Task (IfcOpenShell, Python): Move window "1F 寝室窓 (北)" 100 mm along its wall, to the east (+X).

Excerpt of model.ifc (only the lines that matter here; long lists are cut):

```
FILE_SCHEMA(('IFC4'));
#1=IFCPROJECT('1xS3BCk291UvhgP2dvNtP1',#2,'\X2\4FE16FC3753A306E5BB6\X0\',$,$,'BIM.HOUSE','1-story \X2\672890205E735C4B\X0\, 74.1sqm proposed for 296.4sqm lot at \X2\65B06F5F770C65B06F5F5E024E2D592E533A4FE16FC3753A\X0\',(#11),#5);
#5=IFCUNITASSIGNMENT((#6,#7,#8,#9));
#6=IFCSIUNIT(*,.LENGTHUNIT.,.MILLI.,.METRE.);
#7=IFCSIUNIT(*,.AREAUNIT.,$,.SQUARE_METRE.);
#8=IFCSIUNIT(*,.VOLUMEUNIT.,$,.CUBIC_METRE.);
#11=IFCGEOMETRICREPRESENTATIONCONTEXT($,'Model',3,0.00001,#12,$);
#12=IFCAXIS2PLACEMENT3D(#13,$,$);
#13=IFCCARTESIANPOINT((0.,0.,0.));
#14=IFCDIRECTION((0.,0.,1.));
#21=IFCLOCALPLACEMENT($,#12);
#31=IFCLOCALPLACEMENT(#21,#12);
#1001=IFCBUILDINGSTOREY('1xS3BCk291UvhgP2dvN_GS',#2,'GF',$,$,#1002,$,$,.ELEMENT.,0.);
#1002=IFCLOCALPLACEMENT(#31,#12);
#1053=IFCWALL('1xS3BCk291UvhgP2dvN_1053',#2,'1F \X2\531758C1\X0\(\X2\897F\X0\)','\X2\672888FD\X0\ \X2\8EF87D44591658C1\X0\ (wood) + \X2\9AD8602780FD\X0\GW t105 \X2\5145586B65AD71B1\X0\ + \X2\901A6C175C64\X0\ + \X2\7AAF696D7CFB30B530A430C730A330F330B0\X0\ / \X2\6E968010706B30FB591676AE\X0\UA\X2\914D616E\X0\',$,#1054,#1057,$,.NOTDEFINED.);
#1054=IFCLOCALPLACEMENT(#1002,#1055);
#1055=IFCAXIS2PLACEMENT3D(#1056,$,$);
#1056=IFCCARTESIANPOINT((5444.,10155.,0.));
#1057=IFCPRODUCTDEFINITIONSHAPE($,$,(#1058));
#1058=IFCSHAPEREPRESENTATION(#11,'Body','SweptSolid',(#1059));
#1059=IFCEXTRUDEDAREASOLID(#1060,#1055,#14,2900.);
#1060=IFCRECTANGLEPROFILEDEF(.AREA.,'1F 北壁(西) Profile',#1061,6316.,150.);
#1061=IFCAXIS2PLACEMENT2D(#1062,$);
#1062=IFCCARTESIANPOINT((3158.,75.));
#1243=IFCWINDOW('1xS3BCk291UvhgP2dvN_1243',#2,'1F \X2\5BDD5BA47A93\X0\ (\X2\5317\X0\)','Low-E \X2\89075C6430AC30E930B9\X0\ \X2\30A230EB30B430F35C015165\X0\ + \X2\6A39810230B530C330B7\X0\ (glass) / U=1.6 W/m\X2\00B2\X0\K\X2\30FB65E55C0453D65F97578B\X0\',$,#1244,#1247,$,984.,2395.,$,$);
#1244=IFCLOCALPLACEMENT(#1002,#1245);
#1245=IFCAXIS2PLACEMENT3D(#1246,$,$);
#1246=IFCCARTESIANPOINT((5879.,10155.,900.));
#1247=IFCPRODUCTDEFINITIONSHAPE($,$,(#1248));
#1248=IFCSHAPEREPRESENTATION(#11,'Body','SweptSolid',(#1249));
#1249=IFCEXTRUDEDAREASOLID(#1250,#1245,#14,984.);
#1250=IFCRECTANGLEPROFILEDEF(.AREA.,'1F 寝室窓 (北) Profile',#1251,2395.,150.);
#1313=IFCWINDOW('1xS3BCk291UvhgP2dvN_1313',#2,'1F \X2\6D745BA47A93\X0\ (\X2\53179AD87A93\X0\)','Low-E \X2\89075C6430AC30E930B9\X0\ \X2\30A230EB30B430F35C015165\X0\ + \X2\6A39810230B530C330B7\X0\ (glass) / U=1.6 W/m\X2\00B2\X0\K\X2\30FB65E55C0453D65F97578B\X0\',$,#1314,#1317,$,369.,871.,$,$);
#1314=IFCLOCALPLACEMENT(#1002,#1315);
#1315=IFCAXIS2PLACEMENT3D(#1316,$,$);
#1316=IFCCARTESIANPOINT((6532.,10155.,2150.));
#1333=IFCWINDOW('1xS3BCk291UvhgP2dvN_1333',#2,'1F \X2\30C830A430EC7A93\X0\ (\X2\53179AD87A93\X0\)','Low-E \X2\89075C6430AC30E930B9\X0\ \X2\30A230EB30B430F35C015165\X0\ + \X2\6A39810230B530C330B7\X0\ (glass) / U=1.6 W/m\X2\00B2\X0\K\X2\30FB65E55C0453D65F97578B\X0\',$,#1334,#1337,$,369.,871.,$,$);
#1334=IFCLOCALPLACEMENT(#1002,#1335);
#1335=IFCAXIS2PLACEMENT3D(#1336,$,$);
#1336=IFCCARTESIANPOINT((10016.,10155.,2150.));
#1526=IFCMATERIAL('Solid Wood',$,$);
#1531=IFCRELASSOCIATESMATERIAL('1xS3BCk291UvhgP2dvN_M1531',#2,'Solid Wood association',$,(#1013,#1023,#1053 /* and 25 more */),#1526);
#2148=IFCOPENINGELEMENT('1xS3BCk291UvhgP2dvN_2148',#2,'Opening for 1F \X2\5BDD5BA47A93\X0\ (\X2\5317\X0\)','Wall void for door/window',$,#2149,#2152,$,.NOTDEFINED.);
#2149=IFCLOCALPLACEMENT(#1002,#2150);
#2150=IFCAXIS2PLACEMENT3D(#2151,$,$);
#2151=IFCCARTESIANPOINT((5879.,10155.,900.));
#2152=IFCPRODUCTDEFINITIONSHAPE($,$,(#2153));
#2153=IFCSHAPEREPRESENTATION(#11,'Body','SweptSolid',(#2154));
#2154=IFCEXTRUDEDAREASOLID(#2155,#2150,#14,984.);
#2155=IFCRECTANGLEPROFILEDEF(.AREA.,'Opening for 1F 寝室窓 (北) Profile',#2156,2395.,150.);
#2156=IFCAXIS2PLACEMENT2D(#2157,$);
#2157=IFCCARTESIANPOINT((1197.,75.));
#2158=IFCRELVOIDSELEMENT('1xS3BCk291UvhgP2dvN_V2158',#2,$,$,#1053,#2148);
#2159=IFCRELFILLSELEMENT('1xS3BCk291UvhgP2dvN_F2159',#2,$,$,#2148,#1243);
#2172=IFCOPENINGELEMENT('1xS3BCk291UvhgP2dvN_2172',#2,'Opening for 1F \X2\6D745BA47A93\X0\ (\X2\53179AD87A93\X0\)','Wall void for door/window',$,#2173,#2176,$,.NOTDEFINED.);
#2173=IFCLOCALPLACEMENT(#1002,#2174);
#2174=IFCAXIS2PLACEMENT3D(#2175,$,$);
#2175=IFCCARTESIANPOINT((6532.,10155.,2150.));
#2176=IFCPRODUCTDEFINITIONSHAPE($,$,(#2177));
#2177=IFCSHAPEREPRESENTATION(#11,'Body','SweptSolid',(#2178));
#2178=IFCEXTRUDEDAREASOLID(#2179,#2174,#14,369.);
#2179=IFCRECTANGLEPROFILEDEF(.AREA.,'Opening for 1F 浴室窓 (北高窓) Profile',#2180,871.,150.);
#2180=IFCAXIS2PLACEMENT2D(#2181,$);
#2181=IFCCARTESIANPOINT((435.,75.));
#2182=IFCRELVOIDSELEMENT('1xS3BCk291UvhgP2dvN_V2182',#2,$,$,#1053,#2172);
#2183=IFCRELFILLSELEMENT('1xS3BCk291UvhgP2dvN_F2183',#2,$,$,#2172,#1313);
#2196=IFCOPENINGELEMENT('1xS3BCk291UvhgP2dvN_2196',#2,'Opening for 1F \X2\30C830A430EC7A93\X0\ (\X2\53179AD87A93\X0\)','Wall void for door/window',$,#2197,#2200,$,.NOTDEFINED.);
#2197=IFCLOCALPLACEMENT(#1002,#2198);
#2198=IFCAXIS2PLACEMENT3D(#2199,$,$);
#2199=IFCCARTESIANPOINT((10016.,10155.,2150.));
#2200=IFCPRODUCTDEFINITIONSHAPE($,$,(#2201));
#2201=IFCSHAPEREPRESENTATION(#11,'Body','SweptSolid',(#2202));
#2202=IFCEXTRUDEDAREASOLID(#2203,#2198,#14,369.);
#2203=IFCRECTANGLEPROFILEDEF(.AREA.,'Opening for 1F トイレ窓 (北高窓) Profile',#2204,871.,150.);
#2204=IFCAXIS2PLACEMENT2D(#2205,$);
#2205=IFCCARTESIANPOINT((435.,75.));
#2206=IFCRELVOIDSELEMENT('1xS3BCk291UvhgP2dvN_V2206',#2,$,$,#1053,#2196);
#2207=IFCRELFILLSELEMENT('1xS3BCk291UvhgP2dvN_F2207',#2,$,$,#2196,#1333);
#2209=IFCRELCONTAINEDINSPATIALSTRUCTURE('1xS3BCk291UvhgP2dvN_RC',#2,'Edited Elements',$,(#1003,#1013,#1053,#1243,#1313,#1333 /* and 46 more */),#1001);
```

```python
import ifcopenshell
import ifcopenshell.api.geometry
import ifcopenshell.util.placement
import ifcopenshell.util.unit

model = ifcopenshell.open("model.ifc")
unit_scale = ifcopenshell.util.unit.calculate_unit_scale(model)

window = model.by_id(1243)
opening = window.FillsVoids[0].RelatingOpeningElement
wall = opening.VoidsElements[0].RelatingBuildingElement

wall_matrix = ifcopenshell.util.placement.get_local_placement(wall.ObjectPlacement)
shift = wall_matrix[:3, 0] * 0.1 / unit_scale
before = ifcopenshell.util.placement.get_local_placement(window.ObjectPlacement)[:3, 3].copy()

# The window is not placed relative to its opening, so move both.
for product in (opening, window):
    matrix = ifcopenshell.util.placement.get_local_placement(product.ObjectPlacement)
    matrix[:3, 3] += shift
    ifcopenshell.api.geometry.edit_object_placement(model, product=product, matrix=matrix, is_si=False)

after = ifcopenshell.util.placement.get_local_placement(window.ObjectPlacement)[:3, 3]
print("window moved by", (after - before).round(3) + 0.0)

model.write("model_updated.ifc")
```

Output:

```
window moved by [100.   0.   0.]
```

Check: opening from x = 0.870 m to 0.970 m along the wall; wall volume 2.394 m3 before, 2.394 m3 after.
